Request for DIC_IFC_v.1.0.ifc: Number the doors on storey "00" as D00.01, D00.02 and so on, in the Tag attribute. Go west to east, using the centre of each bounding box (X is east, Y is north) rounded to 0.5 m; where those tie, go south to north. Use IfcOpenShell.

First a look at what the model holds.

```python
import ifcopenshell
import ifcopenshell.util.element
import ifcopenshell.util.placement

model = ifcopenshell.open("DIC_IFC_v.1.0.ifc")
print(model.schema)
storey = next(s for s in model.by_type("IfcBuildingStorey") if s.Name == "00")
doors = [e for e in ifcopenshell.util.element.get_decomposition(storey) if e.is_a("IfcDoor")]
for e in sorted(doors, key=lambda e: e.id()):
    origin = ifcopenshell.util.placement.get_local_placement(e.ObjectPlacement)[:3, 3]
    print(e.id(), e.Tag, e.Name, origin.round(2) + 0.0, sep=" | ")
```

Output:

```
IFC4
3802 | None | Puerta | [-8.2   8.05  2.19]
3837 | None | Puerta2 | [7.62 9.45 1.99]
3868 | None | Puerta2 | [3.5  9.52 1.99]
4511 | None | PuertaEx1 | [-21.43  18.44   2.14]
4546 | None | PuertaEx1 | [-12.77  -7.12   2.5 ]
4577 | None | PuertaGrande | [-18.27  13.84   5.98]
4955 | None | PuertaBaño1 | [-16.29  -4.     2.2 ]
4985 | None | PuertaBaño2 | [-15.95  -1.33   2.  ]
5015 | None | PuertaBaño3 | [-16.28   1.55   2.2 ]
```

```python
import ifcopenshell
import ifcopenshell.geom
import ifcopenshell.util.element
import ifcopenshell.util.shape

model = ifcopenshell.open("DIC_IFC_v.1.0.ifc")
settings = ifcopenshell.geom.settings()
settings.set("use-world-coords", True)


def centre(element):
    shape = ifcopenshell.geom.create_shape(settings, element)
    return ifcopenshell.util.shape.get_bbox_centroid(shape.geometry)


storey = next(s for s in model.by_type("IfcBuildingStorey") if s.Name == "00")
doors = [e for e in ifcopenshell.util.element.get_decomposition(storey) if e.is_a("IfcDoor")]

# Insertion points can sit at a corner or the storey origin, so sort by the geometry (in metres).
centres = {e: centre(e) for e in doors}
doors.sort(key=lambda e: (round(centres[e][0] / 0.5), centres[e][1]))

for i, e in enumerate(doors, start=1):
    number = f"D00.{i:02d}"
    e.Tag = number
    print(e.id(), number)

model.write("DIC_IFC_v.1.0-out.ifc")
```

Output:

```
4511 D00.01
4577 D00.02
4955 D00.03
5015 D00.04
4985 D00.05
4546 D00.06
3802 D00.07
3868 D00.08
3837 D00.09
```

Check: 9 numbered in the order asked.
